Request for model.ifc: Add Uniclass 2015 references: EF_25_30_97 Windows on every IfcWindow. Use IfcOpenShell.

First a look at what the model holds.

```python
import ifcopenshell

model = ifcopenshell.open("model.ifc")
print(model.schema)
print("classifications:", [c.Name for c in model.by_type("IfcClassification")])
for ifc_class in ("IfcDoor", "IfcRoof", "IfcStair", "IfcWall", "IfcWindow"):
    print(ifc_class, len(model.by_type(ifc_class)))
```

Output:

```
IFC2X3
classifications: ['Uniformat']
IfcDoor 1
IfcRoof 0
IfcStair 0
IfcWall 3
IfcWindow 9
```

```python
import ifcopenshell
import ifcopenshell.api.classification

model = ifcopenshell.open("model.ifc")

# IFC2X3 requires Source and Edition and has no link from the project to the system.
system = model.create_entity("IfcClassification", Source="NBS", Edition="2015", Name="Uniclass 2015")

codes = {
    "IfcWindow": ("EF_25_30_97", "Windows"),
}
for ifc_class, (code, name) in codes.items():
    products = model.by_type(ifc_class)
    ifcopenshell.api.classification.add_reference(
        model, products=products, classification=system, identification=code, name=name
    )
    print(code, len(products))

model.write("model_edited.ifc")
```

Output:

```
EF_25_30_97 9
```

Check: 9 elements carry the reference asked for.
